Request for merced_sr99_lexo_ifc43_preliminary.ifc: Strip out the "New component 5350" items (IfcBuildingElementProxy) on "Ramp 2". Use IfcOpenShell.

First a look at what the model holds.

```python
import ifcopenshell
import ifcopenshell.util.element

model = ifcopenshell.open("merced_sr99_lexo_ifc43_preliminary.ifc")
print(model.schema)
storey = next(s for s in model.by_type("IfcBuildingStorey") if s.Name == "Ramp 2")
proxies = [e for e in ifcopenshell.util.element.get_decomposition(storey) if e.is_a("IfcBuildingElementProxy")]
seen = {}
for e in proxies:
    element_type = ifcopenshell.util.element.get_type(e)
    name = element_type.Name if element_type not in (None, e) else None
    seen[name] = seen.get(name, 0) + 1
for name, count in sorted(seen.items(), key=str):
    print(count, "x", name)
```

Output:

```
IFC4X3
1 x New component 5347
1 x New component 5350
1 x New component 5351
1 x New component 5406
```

```python
import ifcopenshell
import ifcopenshell.api.root
import ifcopenshell.util.element

model = ifcopenshell.open("merced_sr99_lexo_ifc43_preliminary.ifc")

storey = next(s for s in model.by_type("IfcBuildingStorey") if s.Name == "Ramp 2")
proxies = [e for e in ifcopenshell.util.element.get_decomposition(storey) if e.is_a("IfcBuildingElementProxy")]
targets = [e for e in proxies if (t := ifcopenshell.util.element.get_type(e)) not in (None, e) and t.Name == "New component 5350"]

for e in targets:
    ifcopenshell.api.root.remove_product(model, product=e)
print(len(targets), "removed")

model.write("merced_sr99_lexo_ifc43_preliminary_v2.ifc")
```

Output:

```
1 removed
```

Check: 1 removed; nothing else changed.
